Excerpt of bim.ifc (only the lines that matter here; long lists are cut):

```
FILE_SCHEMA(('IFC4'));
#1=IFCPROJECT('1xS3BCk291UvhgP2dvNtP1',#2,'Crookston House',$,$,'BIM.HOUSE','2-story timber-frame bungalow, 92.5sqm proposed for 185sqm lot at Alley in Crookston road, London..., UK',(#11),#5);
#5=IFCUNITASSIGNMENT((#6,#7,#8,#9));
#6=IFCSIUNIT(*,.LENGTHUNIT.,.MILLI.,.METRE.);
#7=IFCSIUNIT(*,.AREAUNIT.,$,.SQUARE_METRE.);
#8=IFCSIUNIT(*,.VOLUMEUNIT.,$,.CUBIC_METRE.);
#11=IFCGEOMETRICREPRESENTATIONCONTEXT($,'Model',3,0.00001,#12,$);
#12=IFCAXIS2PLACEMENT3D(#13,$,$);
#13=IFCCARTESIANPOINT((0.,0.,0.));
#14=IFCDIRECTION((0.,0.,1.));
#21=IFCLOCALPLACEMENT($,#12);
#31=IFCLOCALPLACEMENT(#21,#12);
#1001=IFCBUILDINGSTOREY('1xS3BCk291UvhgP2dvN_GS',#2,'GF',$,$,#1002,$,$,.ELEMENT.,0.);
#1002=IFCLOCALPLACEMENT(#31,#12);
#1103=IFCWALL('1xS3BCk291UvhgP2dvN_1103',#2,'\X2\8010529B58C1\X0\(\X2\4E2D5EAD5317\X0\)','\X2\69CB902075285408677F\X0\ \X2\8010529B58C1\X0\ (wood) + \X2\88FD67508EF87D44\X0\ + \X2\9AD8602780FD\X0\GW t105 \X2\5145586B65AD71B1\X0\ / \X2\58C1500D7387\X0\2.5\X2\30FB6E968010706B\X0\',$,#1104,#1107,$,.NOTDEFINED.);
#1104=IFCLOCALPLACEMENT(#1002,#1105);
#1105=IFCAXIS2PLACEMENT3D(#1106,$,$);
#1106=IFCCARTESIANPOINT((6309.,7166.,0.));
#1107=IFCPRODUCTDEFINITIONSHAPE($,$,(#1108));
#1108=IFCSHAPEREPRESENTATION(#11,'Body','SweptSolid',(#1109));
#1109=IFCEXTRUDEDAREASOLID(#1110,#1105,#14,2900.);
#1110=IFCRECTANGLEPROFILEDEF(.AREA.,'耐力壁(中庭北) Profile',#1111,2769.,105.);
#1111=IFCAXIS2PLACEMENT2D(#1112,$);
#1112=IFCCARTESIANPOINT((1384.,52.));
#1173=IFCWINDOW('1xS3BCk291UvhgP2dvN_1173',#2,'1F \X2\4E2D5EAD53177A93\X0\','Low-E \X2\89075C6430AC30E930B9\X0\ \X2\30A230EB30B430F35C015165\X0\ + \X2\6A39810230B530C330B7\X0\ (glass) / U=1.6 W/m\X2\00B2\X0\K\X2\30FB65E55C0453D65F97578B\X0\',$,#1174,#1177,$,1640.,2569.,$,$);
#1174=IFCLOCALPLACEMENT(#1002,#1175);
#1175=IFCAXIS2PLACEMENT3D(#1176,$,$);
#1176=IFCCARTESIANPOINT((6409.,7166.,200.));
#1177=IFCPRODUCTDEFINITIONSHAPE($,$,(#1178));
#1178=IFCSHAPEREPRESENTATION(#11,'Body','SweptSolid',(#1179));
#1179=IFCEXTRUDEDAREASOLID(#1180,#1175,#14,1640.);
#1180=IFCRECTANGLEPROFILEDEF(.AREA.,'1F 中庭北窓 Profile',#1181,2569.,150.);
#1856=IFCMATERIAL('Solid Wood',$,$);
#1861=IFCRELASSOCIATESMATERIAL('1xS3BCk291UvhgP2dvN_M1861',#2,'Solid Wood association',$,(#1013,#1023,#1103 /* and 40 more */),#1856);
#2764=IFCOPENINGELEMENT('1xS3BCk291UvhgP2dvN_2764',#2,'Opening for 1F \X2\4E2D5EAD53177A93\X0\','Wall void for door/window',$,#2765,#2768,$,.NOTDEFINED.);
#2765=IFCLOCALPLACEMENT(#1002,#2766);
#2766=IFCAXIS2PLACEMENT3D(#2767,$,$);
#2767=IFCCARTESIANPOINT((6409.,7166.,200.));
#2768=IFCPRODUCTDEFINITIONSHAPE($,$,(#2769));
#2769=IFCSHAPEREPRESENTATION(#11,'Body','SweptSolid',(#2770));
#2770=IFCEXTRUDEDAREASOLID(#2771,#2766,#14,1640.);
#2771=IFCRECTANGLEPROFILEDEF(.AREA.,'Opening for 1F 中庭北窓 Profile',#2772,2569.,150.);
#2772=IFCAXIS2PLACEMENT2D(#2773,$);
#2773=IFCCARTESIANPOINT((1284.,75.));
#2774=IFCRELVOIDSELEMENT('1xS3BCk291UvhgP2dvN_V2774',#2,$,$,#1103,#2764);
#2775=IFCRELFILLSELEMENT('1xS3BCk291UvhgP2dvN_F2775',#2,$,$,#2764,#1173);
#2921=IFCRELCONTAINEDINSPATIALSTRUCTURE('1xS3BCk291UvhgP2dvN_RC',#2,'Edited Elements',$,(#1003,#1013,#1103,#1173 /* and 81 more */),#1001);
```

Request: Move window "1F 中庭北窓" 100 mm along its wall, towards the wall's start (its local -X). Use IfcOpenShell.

```python
import ifcopenshell
import ifcopenshell.api.geometry
import ifcopenshell.util.placement
import ifcopenshell.util.unit

model = ifcopenshell.open("bim.ifc")
unit_scale = ifcopenshell.util.unit.calculate_unit_scale(model)

window = model.by_guid("1xS3BCk291UvhgP2dvN_1173")
opening = window.FillsVoids[0].RelatingOpeningElement
wall = opening.VoidsElements[0].RelatingBuildingElement

wall_matrix = ifcopenshell.util.placement.get_local_placement(wall.ObjectPlacement)
shift = wall_matrix[:3, 0] * -0.1 / unit_scale
before = ifcopenshell.util.placement.get_local_placement(window.ObjectPlacement)[:3, 3].copy()

# The window is not placed relative to its opening, so move both.
for product in (opening, window):
    matrix = ifcopenshell.util.placement.get_local_placement(product.ObjectPlacement)
    matrix[:3, 3] += shift
    ifcopenshell.api.geometry.edit_object_placement(model, product=product, matrix=matrix, is_si=False)

after = ifcopenshell.util.placement.get_local_placement(window.ObjectPlacement)[:3, 3]
print("window moved by", (after - before).round(3) + 0.0)

model.write("bim_rev.ifc")
```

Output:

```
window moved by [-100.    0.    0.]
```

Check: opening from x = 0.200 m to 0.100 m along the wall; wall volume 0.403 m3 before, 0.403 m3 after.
